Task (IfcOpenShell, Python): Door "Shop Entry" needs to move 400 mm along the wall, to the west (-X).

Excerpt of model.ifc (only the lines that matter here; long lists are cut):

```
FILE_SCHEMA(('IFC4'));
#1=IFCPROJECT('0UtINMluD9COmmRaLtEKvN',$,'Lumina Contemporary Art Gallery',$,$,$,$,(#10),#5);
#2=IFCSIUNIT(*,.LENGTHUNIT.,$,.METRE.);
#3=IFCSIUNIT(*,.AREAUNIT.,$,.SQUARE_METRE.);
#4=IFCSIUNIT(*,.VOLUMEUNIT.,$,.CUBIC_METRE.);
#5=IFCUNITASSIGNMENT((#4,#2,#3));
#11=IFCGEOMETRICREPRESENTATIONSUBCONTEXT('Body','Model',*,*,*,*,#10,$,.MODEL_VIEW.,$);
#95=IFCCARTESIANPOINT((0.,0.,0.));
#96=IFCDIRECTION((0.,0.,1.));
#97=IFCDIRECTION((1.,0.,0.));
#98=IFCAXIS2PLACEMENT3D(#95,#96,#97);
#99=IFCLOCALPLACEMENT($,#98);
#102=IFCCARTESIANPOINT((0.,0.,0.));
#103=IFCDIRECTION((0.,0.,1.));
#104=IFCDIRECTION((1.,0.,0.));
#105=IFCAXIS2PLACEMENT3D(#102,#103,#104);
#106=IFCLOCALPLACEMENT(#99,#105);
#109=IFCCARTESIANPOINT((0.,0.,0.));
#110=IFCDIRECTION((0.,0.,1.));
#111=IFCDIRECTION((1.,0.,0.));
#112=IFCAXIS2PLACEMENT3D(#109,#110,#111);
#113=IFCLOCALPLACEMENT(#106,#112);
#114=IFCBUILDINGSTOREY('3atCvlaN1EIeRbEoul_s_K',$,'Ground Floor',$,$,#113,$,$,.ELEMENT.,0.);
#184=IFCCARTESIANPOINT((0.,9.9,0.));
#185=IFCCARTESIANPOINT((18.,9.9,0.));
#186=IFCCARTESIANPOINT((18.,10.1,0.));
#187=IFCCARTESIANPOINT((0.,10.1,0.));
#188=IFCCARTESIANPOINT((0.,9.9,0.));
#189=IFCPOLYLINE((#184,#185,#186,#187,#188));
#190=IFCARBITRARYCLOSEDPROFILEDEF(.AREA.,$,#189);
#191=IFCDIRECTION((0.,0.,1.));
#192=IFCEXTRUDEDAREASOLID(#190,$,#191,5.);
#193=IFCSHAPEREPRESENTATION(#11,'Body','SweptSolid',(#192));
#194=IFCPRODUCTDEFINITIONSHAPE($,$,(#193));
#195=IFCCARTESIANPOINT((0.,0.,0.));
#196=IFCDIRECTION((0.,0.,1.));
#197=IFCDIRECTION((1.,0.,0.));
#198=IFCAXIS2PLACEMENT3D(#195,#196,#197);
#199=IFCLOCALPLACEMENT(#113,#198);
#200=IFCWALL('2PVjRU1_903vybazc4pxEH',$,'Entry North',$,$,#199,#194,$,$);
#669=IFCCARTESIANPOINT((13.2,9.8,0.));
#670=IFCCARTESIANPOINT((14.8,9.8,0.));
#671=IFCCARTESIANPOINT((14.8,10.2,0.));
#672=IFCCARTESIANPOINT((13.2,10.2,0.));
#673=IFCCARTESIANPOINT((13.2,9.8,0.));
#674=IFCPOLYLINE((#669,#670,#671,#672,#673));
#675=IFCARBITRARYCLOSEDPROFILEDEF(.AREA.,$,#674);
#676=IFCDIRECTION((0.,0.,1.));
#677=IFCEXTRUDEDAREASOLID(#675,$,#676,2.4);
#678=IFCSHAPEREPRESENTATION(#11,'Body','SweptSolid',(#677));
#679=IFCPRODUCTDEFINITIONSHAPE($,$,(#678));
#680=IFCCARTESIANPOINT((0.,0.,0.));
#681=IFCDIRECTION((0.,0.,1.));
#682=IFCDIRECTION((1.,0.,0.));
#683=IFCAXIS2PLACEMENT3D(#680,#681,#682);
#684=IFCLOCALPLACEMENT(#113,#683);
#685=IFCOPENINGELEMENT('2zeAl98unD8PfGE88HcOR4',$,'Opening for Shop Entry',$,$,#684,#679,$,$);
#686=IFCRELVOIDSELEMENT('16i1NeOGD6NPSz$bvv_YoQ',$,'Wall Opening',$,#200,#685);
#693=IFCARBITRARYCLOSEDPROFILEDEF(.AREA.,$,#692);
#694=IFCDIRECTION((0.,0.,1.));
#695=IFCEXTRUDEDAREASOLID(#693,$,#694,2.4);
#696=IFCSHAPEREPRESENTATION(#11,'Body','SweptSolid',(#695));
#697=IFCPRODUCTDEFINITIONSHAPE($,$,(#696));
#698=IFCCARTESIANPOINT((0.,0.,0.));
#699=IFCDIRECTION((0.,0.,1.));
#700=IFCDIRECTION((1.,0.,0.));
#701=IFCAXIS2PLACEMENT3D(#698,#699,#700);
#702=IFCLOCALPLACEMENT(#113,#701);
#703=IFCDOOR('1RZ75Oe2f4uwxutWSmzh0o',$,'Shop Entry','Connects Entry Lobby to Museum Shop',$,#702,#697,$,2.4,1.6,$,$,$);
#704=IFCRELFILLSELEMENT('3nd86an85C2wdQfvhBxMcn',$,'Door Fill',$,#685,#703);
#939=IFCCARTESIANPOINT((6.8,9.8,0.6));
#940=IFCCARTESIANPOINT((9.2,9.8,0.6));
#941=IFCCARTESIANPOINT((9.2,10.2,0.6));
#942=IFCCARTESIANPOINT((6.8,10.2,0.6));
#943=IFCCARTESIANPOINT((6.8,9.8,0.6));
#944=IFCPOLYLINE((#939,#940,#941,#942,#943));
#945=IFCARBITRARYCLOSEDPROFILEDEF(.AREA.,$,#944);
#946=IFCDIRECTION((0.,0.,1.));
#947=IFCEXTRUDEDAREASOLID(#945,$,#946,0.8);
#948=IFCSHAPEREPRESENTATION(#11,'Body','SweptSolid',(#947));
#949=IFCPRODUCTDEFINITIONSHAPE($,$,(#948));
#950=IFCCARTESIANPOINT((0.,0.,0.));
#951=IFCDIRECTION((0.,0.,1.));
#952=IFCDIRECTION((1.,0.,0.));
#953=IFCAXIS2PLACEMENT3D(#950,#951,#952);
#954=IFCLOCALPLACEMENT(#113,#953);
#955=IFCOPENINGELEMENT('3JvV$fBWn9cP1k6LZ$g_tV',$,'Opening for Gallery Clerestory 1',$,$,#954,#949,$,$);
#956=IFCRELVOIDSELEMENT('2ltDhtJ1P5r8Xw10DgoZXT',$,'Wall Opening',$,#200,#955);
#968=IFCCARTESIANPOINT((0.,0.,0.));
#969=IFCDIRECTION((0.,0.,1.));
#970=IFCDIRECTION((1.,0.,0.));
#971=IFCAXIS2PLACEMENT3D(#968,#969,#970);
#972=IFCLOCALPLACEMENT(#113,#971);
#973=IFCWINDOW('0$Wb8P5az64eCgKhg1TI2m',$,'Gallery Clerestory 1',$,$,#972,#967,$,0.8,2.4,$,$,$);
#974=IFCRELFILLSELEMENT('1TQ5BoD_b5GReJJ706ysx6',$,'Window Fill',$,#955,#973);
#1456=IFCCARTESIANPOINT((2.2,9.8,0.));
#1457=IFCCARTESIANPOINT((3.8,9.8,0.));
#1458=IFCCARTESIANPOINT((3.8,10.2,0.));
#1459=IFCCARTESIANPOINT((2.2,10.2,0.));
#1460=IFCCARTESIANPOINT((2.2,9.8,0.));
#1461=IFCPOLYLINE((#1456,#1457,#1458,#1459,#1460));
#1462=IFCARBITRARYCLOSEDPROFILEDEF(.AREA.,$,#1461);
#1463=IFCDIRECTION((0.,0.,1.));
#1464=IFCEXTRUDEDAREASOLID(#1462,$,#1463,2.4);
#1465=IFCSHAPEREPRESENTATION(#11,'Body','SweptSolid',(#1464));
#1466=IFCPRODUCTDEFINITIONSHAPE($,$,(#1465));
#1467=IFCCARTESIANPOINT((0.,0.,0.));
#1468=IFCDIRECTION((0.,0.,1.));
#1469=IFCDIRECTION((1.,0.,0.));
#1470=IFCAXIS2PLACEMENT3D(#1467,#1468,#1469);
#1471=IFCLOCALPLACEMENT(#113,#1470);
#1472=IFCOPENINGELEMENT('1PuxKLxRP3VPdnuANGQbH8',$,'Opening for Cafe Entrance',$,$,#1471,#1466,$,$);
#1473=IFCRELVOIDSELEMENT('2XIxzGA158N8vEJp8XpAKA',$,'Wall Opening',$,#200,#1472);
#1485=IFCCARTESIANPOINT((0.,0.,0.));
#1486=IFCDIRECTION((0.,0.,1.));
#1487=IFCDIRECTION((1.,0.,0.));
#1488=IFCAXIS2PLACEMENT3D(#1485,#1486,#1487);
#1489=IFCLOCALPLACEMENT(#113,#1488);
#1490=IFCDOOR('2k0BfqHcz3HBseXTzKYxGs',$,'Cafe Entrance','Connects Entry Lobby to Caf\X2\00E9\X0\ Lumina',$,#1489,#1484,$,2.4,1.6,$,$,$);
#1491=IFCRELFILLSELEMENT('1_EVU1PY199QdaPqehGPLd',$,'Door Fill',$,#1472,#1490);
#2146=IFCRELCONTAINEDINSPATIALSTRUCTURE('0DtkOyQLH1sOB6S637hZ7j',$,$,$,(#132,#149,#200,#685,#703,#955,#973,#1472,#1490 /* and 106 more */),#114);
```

```python
import ifcopenshell
import ifcopenshell.api.geometry
import ifcopenshell.util.placement
import ifcopenshell.util.unit

model = ifcopenshell.open("model.ifc")
unit_scale = ifcopenshell.util.unit.calculate_unit_scale(model)

door = model.by_guid("1RZ75Oe2f4uwxutWSmzh0o")
opening = door.FillsVoids[0].RelatingOpeningElement
wall = opening.VoidsElements[0].RelatingBuildingElement

wall_matrix = ifcopenshell.util.placement.get_local_placement(wall.ObjectPlacement)
shift = wall_matrix[:3, 0] * -0.4 / unit_scale
before = ifcopenshell.util.placement.get_local_placement(door.ObjectPlacement)[:3, 3].copy()

# The door is not placed relative to its opening, so move both.
for product in (opening, door):
    matrix = ifcopenshell.util.placement.get_local_placement(product.ObjectPlacement)
    matrix[:3, 3] += shift
    ifcopenshell.api.geometry.edit_object_placement(model, product=product, matrix=matrix, is_si=False)

after = ifcopenshell.util.placement.get_local_placement(door.ObjectPlacement)[:3, 3]
print("door moved by", (after - before).round(3) + 0.0)

model.write("model-out.ifc")
```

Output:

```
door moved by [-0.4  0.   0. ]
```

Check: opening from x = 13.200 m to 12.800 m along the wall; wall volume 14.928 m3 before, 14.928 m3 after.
